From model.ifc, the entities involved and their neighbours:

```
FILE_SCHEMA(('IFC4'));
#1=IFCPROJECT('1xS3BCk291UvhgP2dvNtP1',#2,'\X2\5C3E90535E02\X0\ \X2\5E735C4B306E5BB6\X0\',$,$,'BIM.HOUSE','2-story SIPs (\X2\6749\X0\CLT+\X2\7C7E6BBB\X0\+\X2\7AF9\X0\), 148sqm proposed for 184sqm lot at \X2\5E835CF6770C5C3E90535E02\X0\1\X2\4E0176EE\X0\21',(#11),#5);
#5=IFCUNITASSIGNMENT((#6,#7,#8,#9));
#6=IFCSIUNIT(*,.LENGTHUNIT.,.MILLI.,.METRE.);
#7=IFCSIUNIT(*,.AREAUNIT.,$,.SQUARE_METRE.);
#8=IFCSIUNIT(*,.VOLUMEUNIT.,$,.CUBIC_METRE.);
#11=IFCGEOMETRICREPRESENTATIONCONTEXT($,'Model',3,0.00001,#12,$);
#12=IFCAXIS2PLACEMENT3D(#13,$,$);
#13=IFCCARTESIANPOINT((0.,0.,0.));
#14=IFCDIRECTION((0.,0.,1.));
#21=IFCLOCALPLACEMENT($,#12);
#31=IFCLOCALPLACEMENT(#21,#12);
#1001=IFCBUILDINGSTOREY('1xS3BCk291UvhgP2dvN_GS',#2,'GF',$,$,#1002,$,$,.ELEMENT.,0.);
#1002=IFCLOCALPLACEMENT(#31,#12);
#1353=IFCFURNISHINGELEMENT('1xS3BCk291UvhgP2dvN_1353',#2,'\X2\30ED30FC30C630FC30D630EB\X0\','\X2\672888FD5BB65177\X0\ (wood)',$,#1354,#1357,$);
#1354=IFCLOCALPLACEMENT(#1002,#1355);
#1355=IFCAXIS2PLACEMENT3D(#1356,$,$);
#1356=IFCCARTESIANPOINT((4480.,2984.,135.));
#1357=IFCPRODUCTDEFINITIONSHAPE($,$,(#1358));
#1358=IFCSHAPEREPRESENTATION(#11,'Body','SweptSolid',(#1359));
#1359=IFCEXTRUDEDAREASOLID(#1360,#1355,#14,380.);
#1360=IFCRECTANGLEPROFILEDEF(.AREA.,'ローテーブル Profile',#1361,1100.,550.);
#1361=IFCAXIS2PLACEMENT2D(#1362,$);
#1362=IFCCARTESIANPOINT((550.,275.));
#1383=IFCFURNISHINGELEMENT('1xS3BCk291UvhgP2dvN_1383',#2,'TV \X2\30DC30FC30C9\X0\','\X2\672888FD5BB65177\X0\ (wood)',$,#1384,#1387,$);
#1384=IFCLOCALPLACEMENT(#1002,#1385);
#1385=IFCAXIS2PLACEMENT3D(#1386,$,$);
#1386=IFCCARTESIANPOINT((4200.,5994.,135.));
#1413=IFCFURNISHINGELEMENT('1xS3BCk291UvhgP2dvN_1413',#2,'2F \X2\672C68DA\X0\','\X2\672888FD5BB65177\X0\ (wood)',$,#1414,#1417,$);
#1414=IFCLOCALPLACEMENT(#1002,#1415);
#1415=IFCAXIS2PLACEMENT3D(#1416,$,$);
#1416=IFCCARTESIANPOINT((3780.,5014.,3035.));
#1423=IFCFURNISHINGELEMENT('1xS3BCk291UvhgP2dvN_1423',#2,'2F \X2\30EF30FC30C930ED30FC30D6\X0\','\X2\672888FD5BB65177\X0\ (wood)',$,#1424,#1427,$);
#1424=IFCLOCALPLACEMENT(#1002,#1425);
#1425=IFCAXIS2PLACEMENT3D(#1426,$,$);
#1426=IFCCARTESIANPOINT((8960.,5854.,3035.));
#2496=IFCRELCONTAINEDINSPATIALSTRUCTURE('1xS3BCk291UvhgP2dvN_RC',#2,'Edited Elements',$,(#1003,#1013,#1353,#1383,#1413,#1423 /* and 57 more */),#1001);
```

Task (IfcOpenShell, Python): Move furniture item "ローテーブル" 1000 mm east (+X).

```python
import ifcopenshell
import ifcopenshell.api.geometry
import ifcopenshell.util.placement

model = ifcopenshell.open("model.ifc")

item = model.by_id(1353)
matrix = ifcopenshell.util.placement.get_local_placement(item.ObjectPlacement)
matrix[0, 3] += 1000.0
ifcopenshell.api.geometry.edit_object_placement(model, product=item, matrix=matrix, is_si=False)

print(ifcopenshell.util.placement.get_local_placement(item.ObjectPlacement).round(3) + 0.0)

model.write("model_v2.ifc")
```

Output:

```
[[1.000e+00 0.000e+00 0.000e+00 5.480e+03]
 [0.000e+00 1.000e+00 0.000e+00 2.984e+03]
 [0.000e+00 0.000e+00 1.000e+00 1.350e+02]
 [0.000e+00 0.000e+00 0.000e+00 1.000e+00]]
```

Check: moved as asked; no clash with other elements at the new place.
